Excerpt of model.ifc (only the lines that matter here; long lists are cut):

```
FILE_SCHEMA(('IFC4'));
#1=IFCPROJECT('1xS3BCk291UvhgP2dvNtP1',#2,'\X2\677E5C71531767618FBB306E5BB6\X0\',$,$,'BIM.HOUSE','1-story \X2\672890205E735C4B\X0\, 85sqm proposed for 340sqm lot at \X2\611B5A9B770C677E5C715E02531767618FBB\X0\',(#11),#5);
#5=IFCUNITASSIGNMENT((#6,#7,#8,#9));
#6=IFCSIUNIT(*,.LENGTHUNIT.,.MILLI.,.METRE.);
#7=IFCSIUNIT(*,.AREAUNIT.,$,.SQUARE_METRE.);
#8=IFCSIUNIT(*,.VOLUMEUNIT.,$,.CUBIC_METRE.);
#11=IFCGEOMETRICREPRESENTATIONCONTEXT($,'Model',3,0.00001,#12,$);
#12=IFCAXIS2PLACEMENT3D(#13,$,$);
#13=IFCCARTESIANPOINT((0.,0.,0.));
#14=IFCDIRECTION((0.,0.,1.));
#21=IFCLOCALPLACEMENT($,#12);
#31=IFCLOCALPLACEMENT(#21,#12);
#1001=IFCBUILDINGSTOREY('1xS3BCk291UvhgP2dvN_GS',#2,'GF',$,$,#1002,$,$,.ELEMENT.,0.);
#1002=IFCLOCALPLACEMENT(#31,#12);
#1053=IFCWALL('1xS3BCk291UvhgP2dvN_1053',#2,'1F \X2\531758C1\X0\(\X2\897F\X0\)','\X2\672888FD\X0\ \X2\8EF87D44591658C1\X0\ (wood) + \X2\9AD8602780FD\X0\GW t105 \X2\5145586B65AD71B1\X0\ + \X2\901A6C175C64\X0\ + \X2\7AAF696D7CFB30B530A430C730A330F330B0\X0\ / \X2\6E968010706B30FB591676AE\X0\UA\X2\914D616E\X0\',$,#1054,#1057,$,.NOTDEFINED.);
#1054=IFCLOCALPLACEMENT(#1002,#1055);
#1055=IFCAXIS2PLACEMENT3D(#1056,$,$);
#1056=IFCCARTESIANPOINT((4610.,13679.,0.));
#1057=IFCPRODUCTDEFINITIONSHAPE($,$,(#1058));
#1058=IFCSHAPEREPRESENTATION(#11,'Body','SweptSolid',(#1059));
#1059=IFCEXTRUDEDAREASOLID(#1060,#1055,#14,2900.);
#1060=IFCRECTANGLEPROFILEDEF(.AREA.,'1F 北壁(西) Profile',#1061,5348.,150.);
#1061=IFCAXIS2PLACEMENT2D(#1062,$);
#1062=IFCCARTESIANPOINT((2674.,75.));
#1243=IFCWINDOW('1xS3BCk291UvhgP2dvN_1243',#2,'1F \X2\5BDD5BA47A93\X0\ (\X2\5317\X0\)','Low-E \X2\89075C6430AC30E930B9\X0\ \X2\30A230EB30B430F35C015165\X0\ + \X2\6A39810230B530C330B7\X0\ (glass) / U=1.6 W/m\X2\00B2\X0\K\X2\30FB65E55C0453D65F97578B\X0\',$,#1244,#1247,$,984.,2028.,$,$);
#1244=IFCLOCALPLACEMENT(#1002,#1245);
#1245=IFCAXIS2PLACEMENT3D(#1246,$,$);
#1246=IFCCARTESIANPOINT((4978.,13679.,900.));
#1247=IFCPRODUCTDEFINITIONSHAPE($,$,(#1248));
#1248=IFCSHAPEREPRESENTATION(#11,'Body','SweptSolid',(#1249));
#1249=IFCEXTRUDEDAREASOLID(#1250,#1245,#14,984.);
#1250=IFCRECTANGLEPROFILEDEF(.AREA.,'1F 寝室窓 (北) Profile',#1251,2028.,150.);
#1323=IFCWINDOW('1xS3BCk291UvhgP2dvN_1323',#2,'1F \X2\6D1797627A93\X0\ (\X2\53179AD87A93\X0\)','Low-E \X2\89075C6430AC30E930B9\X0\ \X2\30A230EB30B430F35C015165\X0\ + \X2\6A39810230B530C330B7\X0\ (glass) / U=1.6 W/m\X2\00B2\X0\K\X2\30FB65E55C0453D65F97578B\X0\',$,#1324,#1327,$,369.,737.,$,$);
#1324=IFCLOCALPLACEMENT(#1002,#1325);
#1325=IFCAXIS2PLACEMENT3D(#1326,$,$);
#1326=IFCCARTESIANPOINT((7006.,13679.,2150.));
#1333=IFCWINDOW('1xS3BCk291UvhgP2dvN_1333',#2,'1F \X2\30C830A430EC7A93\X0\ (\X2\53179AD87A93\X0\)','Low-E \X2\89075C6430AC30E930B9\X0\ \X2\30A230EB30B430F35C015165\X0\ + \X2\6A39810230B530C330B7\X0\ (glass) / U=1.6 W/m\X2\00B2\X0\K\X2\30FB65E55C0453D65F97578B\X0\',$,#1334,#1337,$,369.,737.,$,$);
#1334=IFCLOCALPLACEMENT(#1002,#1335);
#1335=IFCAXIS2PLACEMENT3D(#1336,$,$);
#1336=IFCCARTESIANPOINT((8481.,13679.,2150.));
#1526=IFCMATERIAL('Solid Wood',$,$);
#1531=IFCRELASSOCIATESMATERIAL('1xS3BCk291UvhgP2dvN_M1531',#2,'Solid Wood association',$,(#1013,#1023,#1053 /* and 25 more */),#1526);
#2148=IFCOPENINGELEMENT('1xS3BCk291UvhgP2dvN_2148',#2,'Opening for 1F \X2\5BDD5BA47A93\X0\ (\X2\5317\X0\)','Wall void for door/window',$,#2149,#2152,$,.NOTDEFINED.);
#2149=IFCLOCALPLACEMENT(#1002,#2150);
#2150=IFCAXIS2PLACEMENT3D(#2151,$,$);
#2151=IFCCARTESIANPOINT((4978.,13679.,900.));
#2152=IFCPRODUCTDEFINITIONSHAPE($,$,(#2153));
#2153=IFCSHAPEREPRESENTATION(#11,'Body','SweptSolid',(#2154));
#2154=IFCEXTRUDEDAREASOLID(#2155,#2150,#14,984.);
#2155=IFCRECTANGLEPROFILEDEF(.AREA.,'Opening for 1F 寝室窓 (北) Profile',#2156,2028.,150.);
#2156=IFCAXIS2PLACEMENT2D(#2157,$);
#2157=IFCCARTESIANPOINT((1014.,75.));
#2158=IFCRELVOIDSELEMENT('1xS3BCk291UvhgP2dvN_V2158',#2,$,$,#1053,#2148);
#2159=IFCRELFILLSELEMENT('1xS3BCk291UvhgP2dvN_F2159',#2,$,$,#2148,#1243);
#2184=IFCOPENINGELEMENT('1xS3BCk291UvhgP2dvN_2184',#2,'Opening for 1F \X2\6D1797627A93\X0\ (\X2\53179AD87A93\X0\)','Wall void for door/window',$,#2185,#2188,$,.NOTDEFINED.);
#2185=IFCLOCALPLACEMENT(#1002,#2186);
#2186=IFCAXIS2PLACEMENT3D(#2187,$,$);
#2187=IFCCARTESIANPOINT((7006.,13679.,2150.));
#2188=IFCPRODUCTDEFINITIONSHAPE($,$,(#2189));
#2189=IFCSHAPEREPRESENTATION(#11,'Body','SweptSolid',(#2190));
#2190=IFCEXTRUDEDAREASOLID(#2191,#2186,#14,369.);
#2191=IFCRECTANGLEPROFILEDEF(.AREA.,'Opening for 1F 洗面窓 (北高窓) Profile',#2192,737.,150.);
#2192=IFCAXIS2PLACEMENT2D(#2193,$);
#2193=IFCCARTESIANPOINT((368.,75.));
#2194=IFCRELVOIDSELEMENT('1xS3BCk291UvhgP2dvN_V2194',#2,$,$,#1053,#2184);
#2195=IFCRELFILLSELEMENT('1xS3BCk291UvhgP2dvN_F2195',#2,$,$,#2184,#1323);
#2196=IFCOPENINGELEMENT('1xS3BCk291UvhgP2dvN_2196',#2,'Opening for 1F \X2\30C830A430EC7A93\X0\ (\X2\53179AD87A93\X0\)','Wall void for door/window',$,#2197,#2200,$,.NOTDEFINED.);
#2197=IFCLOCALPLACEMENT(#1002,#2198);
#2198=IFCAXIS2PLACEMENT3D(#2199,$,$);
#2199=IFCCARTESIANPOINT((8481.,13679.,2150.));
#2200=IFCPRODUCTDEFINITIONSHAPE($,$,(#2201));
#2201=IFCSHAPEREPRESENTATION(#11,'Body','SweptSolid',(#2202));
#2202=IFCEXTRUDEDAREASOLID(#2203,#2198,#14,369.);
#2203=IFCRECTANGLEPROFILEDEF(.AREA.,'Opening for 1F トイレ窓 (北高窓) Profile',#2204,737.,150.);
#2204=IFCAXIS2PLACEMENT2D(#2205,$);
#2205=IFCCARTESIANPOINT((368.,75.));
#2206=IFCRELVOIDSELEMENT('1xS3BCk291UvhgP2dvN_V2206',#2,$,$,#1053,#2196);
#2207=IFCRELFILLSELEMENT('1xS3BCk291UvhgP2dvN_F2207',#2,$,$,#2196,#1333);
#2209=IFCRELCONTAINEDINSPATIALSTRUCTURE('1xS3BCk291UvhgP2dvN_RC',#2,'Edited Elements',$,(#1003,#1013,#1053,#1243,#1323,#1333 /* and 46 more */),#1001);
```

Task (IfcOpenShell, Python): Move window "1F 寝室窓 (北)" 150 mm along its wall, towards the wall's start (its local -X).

```python
import ifcopenshell
import ifcopenshell.api.geometry
import ifcopenshell.util.placement

model = ifcopenshell.open("model.ifc")

window = model.by_guid("1xS3BCk291UvhgP2dvN_1243")
opening = window.FillsVoids[0].RelatingOpeningElement
wall = opening.VoidsElements[0].RelatingBuildingElement

wall_matrix = ifcopenshell.util.placement.get_local_placement(wall.ObjectPlacement)
shift = wall_matrix[:3, 0] * -150.0
before = ifcopenshell.util.placement.get_local_placement(window.ObjectPlacement)[:3, 3].copy()

# The window is not placed relative to its opening, so move both.
for product in (opening, window):
    matrix = ifcopenshell.util.placement.get_local_placement(product.ObjectPlacement)
    matrix[:3, 3] += shift
    ifcopenshell.api.geometry.edit_object_placement(model, product=product, matrix=matrix, is_si=False)

after = ifcopenshell.util.placement.get_local_placement(window.ObjectPlacement)[:3, 3]
print("window moved by", (after - before).round(3) + 0.0)

model.write("model_v2.ifc")
```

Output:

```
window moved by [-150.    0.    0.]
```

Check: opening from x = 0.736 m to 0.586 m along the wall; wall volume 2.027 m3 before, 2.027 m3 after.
